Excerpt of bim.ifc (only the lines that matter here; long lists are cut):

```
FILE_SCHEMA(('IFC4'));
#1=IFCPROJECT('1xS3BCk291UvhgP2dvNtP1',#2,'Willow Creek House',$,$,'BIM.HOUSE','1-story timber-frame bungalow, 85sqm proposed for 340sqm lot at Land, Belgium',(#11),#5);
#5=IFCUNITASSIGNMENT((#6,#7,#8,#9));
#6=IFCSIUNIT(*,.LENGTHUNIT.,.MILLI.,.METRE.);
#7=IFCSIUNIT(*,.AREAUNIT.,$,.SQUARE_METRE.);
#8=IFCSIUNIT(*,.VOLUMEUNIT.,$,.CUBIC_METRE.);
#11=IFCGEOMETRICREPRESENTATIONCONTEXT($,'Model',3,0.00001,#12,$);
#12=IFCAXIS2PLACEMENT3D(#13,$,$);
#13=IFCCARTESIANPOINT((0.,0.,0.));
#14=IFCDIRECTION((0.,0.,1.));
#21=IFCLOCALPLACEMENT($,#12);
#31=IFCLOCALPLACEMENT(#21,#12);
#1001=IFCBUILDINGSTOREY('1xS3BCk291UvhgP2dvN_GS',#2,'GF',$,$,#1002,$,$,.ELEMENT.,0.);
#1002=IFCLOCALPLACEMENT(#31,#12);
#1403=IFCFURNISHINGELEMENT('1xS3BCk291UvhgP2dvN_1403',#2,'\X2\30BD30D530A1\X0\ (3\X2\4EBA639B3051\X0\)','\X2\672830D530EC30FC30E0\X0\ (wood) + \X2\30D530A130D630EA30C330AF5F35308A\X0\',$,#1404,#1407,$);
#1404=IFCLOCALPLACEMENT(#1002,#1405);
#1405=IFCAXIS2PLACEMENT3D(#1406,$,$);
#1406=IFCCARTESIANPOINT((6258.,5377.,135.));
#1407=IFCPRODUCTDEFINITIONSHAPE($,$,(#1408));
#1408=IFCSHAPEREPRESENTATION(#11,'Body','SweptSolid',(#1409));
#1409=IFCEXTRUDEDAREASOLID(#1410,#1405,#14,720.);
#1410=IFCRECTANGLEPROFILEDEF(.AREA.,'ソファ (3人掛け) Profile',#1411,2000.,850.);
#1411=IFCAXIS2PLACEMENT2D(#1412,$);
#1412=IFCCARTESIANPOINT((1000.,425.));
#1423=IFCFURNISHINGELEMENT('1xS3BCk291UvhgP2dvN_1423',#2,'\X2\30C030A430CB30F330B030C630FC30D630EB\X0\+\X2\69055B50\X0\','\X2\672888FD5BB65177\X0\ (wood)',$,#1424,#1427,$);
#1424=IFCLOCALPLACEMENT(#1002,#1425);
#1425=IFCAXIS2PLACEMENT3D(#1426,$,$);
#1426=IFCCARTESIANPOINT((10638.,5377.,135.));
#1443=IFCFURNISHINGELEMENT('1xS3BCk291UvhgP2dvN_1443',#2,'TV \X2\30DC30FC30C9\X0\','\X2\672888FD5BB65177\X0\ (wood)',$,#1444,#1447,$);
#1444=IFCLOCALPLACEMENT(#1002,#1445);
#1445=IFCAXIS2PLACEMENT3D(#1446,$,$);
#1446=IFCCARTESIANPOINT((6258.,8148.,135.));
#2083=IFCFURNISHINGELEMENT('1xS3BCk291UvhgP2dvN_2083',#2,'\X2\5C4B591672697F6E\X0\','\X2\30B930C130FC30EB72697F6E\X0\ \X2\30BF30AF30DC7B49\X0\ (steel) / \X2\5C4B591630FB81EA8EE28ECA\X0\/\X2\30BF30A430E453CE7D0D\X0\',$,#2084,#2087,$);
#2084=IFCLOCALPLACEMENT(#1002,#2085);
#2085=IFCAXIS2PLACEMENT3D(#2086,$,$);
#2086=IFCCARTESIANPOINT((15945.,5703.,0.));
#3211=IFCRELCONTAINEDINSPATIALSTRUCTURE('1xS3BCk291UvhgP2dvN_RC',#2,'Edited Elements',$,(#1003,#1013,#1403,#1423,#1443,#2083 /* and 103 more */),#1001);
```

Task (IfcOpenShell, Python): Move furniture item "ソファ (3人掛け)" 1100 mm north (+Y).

```python
import ifcopenshell
import ifcopenshell.api.geometry
import ifcopenshell.util.placement

model = ifcopenshell.open("bim.ifc")

item = model.by_guid("1xS3BCk291UvhgP2dvN_1403")
matrix = ifcopenshell.util.placement.get_local_placement(item.ObjectPlacement)
matrix[1, 3] += 1100.0
ifcopenshell.api.geometry.edit_object_placement(model, product=item, matrix=matrix, is_si=False)

print(ifcopenshell.util.placement.get_local_placement(item.ObjectPlacement).round(3) + 0.0)

model.write("bim_rev.ifc")
```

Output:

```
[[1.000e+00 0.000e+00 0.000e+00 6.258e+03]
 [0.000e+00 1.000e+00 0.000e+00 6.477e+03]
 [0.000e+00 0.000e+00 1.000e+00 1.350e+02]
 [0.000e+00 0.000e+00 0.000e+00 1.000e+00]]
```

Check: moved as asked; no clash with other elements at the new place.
